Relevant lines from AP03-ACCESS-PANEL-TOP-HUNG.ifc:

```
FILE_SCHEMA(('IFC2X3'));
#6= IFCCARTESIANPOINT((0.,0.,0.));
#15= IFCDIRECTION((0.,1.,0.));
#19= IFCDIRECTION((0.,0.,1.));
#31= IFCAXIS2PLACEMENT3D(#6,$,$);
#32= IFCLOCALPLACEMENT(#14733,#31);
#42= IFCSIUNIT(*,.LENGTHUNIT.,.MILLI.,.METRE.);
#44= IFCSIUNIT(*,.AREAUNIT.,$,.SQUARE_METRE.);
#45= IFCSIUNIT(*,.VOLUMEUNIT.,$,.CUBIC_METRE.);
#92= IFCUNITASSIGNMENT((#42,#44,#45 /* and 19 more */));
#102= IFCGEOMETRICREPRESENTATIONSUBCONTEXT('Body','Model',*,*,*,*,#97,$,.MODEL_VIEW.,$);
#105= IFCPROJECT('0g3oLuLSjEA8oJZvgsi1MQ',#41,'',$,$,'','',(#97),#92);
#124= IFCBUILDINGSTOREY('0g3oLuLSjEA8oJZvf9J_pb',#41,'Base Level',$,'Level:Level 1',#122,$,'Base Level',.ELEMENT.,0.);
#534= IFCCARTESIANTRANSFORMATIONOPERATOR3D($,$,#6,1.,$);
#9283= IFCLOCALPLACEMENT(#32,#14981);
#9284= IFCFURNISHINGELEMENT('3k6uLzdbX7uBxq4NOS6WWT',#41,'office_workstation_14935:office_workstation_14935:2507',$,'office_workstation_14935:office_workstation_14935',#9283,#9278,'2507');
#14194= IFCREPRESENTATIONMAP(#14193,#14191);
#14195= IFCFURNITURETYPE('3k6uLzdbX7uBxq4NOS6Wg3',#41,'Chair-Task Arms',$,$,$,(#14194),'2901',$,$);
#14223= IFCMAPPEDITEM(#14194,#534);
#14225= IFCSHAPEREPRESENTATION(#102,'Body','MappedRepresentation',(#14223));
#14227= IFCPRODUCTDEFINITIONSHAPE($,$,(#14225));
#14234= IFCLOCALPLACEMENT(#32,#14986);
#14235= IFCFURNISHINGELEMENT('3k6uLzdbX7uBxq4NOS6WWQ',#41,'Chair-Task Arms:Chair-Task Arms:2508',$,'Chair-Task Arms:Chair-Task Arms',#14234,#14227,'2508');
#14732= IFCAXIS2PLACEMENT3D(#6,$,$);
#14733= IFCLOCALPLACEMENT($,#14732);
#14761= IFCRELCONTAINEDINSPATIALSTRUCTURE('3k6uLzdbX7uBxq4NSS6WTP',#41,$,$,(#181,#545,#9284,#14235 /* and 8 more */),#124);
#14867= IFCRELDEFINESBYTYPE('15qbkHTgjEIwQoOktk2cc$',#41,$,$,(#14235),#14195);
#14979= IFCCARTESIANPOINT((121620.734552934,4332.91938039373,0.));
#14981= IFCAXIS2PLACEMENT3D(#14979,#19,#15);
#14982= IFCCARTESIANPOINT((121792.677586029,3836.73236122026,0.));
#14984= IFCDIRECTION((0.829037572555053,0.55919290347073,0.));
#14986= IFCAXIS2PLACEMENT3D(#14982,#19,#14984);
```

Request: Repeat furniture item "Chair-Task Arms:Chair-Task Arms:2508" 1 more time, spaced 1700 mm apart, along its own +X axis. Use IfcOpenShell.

```python
import ifcopenshell
import ifcopenshell.api.geometry
import ifcopenshell.api.root
import ifcopenshell.util.element
import ifcopenshell.util.placement

model = ifcopenshell.open("AP03-ACCESS-PANEL-TOP-HUNG.ifc")


def reuse_history(source, copy):
    """copy_class also copies each property set's owner history, people and application; keep the originals."""
    for rel in copy.IsDefinedBy:
        if rel.is_a("IfcRelDefinesByProperties") and (history := rel.RelatingPropertyDefinition.OwnerHistory):
            rel.RelatingPropertyDefinition.OwnerHistory = source.OwnerHistory
            ifcopenshell.util.element.remove_deep2(model, history)


source = model.by_id(14235)
base = ifcopenshell.util.placement.get_local_placement(source.ObjectPlacement)
step = base[:3, 0] * 1700.0

for i in range(1, 2):
    copy = ifcopenshell.api.root.copy_class(model, product=source)
    copy.Representation = ifcopenshell.util.element.copy_deep(
        model, source.Representation, exclude=["IfcGeometricRepresentationContext", "IfcRepresentationMap"]
    )
    copy.Name = "Chair-Task Arms:Chair-Task Arms"
    copy.Tag = None
    reuse_history(source, copy)
    matrix = base.copy()
    matrix[:3, 3] += i * step
    print("added at", matrix[:3, 3].round(3) + 0.0)
    ifcopenshell.api.geometry.edit_object_placement(model, product=copy, matrix=matrix, is_si=False)

model.write("AP03-ACCESS-PANEL-TOP-HUNG-out.ifc")
```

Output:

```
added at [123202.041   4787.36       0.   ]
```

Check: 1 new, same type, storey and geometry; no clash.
